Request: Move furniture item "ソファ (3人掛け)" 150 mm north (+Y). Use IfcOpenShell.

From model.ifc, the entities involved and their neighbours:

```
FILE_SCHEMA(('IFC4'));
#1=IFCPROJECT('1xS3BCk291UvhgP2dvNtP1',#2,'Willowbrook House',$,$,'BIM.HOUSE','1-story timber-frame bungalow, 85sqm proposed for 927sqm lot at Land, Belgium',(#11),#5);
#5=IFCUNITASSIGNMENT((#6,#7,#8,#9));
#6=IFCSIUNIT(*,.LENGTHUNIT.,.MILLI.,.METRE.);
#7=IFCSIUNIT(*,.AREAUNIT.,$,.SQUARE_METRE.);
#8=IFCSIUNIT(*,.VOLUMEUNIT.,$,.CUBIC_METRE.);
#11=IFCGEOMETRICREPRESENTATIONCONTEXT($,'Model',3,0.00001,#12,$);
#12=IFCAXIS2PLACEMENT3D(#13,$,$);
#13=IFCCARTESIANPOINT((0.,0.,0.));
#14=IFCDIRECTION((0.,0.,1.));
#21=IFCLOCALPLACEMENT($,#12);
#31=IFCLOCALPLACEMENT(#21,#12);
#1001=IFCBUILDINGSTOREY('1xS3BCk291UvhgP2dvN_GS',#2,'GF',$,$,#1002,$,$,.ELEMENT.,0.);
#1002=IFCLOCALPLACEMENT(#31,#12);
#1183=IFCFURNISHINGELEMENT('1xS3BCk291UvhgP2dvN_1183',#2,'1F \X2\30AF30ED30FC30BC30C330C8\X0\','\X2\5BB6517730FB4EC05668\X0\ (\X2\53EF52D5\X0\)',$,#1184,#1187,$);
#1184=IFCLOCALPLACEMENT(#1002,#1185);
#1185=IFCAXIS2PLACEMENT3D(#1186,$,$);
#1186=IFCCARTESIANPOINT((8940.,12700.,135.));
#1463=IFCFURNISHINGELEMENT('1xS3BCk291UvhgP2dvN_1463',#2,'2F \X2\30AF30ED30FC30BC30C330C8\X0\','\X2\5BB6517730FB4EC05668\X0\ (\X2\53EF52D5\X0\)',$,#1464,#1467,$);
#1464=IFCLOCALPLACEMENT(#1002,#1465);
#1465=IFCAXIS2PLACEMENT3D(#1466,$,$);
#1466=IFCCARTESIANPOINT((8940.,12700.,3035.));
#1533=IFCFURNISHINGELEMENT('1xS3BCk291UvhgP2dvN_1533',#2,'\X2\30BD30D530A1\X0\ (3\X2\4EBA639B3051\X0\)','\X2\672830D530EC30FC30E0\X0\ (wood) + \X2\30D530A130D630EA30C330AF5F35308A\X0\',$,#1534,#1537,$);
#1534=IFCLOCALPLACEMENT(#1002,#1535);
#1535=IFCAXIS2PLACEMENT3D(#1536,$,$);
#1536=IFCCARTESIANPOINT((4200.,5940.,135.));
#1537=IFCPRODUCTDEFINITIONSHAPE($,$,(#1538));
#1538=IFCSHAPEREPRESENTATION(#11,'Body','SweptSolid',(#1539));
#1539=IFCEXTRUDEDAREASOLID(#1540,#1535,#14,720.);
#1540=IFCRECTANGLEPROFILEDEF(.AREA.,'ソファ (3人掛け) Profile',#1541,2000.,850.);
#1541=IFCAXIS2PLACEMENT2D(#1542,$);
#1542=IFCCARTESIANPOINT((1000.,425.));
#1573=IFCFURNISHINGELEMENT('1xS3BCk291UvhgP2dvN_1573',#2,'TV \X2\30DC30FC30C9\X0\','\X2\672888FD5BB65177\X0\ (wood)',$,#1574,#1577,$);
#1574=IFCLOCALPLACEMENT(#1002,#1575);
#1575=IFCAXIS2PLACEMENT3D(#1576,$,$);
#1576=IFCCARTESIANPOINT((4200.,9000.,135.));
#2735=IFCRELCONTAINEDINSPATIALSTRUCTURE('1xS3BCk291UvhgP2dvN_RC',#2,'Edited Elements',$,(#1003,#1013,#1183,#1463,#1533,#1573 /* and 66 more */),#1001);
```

```python
import ifcopenshell
import ifcopenshell.api.geometry
import ifcopenshell.util.placement

model = ifcopenshell.open("model.ifc")

item = model.by_guid("1xS3BCk291UvhgP2dvN_1533")
matrix = ifcopenshell.util.placement.get_local_placement(item.ObjectPlacement)
matrix[1, 3] += 150.0
ifcopenshell.api.geometry.edit_object_placement(model, product=item, matrix=matrix, is_si=False)

print(ifcopenshell.util.placement.get_local_placement(item.ObjectPlacement).round(3) + 0.0)

model.write("model_updated.ifc")
```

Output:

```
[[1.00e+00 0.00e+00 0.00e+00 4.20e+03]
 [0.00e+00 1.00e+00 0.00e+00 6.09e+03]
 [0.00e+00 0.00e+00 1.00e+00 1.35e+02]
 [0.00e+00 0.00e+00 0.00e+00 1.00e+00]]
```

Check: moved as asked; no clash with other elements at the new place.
